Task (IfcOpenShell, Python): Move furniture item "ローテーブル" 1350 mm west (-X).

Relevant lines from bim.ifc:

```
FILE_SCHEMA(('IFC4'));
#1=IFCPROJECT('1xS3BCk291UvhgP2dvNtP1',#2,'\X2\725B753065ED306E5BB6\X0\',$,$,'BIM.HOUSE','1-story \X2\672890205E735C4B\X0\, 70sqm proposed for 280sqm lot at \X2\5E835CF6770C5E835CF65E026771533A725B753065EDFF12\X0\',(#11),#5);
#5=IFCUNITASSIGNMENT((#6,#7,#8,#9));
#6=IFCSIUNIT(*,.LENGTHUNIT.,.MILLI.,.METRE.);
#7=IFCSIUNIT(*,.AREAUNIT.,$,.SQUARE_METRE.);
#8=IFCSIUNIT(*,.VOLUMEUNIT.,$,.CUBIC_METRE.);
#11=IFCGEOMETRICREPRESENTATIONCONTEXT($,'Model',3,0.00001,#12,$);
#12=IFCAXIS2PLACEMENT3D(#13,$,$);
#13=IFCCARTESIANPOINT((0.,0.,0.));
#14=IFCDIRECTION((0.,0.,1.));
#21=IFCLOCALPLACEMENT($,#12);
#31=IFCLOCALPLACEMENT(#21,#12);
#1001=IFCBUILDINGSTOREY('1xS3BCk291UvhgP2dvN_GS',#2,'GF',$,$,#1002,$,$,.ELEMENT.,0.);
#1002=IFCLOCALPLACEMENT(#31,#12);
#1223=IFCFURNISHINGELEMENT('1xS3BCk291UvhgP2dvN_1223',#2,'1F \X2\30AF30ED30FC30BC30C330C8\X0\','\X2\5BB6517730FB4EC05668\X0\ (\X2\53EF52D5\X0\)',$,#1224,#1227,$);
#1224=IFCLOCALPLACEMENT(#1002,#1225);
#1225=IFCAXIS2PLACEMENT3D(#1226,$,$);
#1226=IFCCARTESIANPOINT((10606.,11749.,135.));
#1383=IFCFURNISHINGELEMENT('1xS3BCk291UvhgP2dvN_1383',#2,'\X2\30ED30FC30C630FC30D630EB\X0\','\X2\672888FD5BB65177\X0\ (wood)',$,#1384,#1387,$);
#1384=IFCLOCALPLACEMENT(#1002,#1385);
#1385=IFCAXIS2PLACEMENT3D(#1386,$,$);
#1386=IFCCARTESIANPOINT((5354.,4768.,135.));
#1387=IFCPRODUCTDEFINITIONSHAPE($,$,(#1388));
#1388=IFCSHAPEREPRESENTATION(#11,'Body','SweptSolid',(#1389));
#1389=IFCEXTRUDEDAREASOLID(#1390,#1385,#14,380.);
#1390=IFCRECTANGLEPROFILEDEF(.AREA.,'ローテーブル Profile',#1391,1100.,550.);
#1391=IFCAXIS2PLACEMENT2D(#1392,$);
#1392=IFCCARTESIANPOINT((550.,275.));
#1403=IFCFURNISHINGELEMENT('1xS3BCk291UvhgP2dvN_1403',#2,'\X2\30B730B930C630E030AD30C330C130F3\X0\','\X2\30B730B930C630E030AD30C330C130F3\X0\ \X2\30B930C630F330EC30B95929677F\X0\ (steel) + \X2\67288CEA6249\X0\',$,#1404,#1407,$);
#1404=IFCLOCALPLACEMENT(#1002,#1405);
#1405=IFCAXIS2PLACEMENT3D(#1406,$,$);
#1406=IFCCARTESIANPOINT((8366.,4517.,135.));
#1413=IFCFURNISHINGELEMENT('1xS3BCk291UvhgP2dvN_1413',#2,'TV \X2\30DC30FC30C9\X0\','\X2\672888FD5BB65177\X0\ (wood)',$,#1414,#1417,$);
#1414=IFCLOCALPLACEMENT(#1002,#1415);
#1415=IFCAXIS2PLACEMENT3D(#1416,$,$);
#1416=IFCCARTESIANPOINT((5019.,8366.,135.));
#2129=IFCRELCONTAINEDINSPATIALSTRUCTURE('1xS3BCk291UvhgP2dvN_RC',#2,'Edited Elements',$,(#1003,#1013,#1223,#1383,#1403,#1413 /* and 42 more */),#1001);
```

```python
import ifcopenshell
import ifcopenshell.api.geometry
import ifcopenshell.util.placement
import ifcopenshell.util.unit

model = ifcopenshell.open("bim.ifc")
unit_scale = ifcopenshell.util.unit.calculate_unit_scale(model)

item = model.by_guid("1xS3BCk291UvhgP2dvN_1383")
matrix = ifcopenshell.util.placement.get_local_placement(item.ObjectPlacement)
matrix[0, 3] -= 1.35 / unit_scale
ifcopenshell.api.geometry.edit_object_placement(model, product=item, matrix=matrix, is_si=False)

print(ifcopenshell.util.placement.get_local_placement(item.ObjectPlacement).round(3) + 0.0)

model.write("bim_rev.ifc")
```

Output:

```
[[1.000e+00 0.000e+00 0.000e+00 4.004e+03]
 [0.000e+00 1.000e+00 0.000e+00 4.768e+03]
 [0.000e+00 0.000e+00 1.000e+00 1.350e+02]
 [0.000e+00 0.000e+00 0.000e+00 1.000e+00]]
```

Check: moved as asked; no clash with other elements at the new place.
